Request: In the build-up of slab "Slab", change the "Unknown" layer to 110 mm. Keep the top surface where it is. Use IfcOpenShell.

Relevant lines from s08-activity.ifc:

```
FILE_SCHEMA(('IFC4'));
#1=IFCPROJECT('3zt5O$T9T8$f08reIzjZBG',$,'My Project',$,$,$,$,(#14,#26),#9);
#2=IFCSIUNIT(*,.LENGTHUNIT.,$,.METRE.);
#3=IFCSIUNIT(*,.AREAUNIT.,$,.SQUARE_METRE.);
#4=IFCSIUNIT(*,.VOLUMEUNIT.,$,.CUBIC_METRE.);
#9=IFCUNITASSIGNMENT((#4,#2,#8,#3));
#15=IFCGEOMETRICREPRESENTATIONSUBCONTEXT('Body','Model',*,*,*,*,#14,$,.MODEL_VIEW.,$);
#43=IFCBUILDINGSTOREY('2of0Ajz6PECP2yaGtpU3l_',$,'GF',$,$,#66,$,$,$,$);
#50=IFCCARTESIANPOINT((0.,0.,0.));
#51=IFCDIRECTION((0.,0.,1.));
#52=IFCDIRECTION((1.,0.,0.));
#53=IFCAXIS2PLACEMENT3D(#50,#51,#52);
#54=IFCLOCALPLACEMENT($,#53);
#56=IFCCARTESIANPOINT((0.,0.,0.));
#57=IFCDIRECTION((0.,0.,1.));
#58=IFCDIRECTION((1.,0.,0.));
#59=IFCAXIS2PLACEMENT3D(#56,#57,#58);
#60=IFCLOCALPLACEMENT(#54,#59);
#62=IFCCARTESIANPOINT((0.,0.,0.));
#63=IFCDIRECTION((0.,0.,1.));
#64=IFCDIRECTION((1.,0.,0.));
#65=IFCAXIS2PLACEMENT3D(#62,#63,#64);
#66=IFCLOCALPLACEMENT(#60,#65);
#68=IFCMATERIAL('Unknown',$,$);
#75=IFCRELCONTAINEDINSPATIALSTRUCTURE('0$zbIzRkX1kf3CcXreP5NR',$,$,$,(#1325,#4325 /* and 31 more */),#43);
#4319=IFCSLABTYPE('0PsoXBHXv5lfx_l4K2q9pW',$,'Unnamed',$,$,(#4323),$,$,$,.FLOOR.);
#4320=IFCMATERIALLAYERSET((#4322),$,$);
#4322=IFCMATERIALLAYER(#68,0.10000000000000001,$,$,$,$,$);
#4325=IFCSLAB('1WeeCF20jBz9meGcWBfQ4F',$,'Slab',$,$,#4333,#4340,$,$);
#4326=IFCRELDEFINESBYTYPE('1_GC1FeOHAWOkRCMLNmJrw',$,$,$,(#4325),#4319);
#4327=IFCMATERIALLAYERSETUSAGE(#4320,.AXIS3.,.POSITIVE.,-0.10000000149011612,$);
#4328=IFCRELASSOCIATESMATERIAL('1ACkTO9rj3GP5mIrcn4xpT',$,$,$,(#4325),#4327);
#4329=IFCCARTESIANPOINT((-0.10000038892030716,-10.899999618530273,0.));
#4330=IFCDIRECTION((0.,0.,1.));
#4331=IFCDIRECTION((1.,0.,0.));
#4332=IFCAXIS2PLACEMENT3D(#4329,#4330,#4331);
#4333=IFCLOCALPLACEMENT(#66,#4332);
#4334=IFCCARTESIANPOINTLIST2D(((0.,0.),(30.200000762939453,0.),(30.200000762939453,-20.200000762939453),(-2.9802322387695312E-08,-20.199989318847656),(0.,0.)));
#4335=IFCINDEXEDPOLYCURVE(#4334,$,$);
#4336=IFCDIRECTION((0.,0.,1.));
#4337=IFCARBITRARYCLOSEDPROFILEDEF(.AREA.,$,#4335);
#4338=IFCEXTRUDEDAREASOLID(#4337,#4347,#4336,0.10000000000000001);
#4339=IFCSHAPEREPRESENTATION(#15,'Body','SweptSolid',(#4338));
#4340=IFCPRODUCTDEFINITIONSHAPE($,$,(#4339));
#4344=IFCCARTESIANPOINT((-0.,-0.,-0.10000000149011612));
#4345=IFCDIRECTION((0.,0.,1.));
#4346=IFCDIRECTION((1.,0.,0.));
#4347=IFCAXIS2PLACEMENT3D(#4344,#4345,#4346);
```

```python
import ifcopenshell
import ifcopenshell.util.element
import ifcopenshell.util.representation
import ifcopenshell.util.unit

model = ifcopenshell.open("s08-activity.ifc")
unit_scale = ifcopenshell.util.unit.calculate_unit_scale(model)

layer_set = model.by_id(4320)
layer = next(l for l in layer_set.MaterialLayers if l.Material and l.Material.Name == "Unknown")
change = 0.11 / unit_scale - layer.LayerThickness
layer.LayerThickness += change

# Geometry does not follow the layer set by itself.
slabs = [e for e in ifcopenshell.util.element.get_elements_by_material(model, layer_set) if e.is_a("IfcSlab")]
for slab in sorted(slabs, key=lambda e: e.id()):
    body = ifcopenshell.util.representation.get_representation(slab, "Model", "Body")
    solid = body.Items[0]
    old_depth = solid.Depth
    solid.Depth += change
    # Extruded upwards: lower the start of the extrusion so the top stays.
    x, y, z = solid.Position.Location.Coordinates
    solid.Position.Location = model.createIfcCartesianPoint((x, y, z - change))
    print(slab.id(), f"{old_depth:g} -> {solid.Depth:g}")

# The layers are counted up from the underside, which has moved.
for usage in {ifcopenshell.util.element.get_material(slab) for slab in slabs}:
    usage.OffsetFromReferenceLine -= change

model.write("s08-activity-out.ifc")
```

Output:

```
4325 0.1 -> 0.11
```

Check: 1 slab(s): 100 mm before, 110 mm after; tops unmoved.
